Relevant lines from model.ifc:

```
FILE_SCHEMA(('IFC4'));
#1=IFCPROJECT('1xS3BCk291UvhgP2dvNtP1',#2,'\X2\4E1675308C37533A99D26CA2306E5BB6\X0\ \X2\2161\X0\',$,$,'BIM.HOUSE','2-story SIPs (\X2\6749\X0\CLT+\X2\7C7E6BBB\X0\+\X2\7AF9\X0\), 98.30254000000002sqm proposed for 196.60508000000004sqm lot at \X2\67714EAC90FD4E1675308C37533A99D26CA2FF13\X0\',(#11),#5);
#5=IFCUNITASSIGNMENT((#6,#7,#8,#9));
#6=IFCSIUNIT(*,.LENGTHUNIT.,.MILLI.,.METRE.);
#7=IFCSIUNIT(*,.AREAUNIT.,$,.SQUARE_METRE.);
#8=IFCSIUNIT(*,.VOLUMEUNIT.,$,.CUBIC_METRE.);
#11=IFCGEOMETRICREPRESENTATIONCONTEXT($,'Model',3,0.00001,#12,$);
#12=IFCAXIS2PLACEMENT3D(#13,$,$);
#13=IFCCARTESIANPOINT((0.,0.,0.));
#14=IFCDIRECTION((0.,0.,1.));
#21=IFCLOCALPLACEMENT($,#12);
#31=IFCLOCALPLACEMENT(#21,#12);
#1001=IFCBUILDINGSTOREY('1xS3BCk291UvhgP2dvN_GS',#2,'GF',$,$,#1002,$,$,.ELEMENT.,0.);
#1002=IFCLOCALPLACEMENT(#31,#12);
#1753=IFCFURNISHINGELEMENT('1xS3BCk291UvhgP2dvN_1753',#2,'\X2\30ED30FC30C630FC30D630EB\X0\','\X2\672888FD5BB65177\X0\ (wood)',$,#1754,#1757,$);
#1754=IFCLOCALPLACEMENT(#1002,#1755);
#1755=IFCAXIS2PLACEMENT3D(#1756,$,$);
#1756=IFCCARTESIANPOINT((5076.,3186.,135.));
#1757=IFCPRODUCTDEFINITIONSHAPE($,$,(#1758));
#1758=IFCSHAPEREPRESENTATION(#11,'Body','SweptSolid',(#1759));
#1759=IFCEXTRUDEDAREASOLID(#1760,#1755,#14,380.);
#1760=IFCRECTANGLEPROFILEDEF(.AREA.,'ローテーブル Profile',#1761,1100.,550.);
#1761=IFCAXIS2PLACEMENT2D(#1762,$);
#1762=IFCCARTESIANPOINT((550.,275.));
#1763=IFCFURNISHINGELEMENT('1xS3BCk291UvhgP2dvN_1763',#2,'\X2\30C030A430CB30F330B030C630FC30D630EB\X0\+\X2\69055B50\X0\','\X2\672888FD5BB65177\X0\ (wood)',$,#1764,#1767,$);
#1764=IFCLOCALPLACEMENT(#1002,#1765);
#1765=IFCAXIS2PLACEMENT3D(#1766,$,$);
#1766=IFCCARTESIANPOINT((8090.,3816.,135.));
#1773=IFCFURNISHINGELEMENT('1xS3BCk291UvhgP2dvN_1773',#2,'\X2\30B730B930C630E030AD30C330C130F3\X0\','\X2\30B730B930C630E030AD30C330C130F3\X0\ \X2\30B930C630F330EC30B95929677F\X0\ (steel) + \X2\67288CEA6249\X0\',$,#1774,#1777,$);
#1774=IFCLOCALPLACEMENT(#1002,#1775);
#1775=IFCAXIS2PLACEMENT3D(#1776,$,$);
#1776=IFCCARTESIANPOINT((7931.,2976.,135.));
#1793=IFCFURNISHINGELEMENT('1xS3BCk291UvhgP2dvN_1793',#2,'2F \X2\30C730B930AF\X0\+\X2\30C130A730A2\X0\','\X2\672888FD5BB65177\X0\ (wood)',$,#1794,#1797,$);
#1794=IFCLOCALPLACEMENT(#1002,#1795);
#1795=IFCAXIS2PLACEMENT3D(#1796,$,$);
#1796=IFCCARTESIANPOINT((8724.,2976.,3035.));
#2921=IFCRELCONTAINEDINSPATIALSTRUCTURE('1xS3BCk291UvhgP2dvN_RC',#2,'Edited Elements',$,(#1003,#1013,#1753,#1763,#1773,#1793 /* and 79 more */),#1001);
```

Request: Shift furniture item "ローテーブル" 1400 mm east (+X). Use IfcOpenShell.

```python
import ifcopenshell
import ifcopenshell.api.geometry
import ifcopenshell.util.placement
import ifcopenshell.util.unit

model = ifcopenshell.open("model.ifc")
unit_scale = ifcopenshell.util.unit.calculate_unit_scale(model)

item = model.by_guid("1xS3BCk291UvhgP2dvN_1753")
matrix = ifcopenshell.util.placement.get_local_placement(item.ObjectPlacement)
matrix[0, 3] += 1.4 / unit_scale
ifcopenshell.api.geometry.edit_object_placement(model, product=item, matrix=matrix, is_si=False)

print(ifcopenshell.util.placement.get_local_placement(item.ObjectPlacement).round(3) + 0.0)

model.write("model_updated.ifc")
```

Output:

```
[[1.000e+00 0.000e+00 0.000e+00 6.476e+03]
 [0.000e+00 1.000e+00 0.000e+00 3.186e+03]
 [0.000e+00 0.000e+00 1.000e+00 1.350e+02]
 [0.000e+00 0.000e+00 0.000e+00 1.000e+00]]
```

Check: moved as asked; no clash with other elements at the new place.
